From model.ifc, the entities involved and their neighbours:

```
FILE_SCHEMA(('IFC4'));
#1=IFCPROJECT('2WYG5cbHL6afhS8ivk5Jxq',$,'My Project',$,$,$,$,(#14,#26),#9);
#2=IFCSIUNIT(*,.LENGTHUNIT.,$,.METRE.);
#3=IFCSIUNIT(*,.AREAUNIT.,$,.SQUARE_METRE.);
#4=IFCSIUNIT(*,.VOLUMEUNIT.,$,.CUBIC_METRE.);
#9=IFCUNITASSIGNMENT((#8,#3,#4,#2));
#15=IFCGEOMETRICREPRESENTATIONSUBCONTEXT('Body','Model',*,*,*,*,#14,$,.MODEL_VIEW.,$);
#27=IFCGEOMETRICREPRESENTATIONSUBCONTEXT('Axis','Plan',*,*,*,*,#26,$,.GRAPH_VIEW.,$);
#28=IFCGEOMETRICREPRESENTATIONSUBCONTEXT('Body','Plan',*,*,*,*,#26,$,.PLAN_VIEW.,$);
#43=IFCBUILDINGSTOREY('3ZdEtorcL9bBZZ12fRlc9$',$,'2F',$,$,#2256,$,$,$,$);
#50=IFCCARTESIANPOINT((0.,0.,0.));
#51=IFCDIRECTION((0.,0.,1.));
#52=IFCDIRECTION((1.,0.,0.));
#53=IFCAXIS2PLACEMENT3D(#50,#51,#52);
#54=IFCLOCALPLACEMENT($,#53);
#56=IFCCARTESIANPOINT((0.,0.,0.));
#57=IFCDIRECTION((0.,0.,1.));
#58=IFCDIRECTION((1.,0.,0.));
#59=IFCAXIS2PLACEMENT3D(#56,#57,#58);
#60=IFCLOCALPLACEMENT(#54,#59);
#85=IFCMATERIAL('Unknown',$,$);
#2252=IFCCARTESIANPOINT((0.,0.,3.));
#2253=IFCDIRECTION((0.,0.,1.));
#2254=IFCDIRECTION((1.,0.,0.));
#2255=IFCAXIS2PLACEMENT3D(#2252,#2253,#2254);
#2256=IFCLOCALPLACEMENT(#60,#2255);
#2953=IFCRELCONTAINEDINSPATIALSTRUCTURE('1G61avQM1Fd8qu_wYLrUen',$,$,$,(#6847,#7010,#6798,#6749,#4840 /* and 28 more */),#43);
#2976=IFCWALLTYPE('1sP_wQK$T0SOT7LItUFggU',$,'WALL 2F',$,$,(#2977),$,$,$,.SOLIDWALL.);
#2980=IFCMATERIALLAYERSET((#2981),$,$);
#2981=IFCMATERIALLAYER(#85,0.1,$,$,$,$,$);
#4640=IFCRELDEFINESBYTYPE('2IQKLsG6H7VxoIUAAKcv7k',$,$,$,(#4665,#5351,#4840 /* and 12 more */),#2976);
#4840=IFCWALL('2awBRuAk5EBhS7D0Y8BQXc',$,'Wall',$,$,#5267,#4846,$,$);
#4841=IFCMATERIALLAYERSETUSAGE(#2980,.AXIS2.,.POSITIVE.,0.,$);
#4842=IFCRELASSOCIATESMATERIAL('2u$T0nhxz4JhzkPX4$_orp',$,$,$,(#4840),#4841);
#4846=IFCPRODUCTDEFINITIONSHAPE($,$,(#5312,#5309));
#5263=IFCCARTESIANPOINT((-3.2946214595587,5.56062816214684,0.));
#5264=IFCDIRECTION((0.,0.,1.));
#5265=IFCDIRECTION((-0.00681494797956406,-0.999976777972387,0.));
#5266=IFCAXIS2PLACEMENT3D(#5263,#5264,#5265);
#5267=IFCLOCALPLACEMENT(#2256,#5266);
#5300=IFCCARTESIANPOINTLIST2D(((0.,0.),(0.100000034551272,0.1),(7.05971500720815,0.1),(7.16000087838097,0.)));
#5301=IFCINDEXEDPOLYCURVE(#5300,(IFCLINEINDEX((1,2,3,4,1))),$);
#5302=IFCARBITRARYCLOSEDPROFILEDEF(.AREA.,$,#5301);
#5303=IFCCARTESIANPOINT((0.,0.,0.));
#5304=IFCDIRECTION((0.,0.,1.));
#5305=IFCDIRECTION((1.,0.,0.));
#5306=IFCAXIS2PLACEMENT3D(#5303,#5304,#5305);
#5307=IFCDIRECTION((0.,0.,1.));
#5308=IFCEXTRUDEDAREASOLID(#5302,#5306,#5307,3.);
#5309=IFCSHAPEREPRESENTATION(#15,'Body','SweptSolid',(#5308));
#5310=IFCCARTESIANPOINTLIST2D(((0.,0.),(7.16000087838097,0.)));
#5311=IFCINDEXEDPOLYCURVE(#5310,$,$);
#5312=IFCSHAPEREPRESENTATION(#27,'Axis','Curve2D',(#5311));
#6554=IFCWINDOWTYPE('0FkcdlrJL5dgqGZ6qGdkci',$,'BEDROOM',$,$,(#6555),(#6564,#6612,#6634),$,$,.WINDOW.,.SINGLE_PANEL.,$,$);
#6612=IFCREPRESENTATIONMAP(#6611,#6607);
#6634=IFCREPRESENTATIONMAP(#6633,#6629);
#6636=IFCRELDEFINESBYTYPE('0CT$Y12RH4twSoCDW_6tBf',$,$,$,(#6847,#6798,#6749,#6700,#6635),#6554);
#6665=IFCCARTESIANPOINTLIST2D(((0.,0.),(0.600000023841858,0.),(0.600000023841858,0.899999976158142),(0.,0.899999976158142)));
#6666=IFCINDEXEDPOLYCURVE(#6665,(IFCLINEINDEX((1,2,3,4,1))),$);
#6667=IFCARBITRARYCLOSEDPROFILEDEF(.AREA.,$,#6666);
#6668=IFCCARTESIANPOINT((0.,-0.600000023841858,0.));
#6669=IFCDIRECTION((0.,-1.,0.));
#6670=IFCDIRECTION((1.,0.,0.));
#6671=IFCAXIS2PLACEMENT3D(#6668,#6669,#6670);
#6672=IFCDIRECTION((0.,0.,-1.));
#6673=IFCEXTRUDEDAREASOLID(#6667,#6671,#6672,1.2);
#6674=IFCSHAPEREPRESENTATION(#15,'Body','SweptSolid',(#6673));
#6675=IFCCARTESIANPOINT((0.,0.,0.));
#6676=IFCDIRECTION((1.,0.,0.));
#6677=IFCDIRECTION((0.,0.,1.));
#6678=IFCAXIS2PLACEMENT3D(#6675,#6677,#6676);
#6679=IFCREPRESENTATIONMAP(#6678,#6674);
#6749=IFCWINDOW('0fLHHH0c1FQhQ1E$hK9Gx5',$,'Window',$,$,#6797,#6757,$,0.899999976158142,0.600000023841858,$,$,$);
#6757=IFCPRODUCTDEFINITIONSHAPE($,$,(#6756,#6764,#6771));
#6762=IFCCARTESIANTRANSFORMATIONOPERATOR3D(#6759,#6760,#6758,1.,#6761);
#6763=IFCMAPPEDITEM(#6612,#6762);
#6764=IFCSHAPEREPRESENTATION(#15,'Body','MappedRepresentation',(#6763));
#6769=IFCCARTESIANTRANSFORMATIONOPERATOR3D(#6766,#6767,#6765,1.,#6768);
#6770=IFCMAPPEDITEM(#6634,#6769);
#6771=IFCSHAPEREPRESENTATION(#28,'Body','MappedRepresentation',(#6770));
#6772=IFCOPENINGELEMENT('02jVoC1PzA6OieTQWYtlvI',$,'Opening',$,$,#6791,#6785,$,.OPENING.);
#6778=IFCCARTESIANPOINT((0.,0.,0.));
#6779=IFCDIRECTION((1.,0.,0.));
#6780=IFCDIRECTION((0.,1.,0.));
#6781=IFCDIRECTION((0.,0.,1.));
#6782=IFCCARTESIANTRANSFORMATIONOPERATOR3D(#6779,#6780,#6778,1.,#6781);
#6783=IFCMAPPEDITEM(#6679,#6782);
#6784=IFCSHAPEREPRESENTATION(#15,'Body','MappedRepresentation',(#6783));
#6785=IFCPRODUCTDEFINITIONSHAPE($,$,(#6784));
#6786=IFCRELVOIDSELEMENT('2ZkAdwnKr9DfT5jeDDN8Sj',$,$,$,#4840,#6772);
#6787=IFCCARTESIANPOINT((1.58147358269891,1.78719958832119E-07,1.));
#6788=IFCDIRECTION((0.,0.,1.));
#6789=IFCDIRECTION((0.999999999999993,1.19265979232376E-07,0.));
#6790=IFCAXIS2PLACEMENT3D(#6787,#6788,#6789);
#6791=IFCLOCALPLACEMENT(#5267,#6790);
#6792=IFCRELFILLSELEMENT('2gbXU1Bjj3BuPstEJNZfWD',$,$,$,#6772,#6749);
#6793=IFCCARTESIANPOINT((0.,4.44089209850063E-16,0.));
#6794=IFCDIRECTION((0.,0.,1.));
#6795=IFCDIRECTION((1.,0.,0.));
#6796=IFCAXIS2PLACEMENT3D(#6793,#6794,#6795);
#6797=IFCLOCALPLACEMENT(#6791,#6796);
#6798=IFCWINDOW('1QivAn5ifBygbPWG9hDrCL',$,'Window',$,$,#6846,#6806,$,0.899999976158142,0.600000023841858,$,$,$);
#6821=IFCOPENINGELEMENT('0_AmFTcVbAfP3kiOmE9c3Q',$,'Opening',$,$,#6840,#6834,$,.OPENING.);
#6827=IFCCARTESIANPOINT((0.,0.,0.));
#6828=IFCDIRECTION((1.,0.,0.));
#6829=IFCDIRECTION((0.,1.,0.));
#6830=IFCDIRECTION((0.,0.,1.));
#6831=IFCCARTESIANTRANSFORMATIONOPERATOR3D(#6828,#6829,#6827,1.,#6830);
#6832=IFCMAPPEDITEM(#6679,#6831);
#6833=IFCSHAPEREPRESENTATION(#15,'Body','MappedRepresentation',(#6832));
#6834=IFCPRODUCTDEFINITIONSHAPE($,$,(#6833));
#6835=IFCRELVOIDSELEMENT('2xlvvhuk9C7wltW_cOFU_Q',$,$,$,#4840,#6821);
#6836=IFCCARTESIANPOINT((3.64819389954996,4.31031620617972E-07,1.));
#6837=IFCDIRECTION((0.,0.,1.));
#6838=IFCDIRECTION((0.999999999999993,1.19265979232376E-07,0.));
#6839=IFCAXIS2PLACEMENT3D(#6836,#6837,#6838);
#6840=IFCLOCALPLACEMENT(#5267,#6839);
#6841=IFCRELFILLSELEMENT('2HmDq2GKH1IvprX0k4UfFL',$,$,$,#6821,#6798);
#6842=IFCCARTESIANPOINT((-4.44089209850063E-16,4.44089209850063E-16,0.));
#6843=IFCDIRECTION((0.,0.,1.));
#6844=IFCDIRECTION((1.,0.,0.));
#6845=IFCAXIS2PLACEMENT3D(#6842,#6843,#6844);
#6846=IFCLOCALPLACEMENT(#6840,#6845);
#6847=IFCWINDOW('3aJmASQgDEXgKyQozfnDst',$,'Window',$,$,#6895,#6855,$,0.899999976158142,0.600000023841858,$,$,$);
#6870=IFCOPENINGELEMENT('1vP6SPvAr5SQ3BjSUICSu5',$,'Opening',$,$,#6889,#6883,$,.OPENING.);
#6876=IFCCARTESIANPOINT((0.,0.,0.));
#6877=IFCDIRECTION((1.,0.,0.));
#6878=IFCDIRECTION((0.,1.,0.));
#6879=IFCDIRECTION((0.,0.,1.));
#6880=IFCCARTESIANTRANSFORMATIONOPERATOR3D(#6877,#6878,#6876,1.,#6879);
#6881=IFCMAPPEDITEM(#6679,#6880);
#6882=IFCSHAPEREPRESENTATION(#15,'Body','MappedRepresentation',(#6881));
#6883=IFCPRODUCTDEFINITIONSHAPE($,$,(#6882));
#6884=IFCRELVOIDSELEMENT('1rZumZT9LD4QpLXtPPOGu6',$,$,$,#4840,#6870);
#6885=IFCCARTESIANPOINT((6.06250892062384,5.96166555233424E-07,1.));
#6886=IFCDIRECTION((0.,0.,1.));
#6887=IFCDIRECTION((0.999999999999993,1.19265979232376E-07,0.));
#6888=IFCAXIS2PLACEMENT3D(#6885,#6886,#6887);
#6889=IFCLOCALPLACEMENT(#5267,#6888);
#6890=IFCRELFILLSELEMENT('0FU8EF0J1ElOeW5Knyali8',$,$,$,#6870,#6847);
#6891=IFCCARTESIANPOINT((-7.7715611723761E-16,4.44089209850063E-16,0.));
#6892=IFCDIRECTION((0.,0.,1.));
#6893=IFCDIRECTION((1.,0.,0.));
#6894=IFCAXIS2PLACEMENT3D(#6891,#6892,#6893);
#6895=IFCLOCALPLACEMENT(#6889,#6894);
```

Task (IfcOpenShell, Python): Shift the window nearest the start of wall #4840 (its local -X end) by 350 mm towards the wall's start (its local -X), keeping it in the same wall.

```python
import ifcopenshell
import ifcopenshell.api.geometry
import ifcopenshell.util.placement

model = ifcopenshell.open("model.ifc")

window = model.by_id(6749)
opening = window.FillsVoids[0].RelatingOpeningElement
wall = opening.VoidsElements[0].RelatingBuildingElement

wall_matrix = ifcopenshell.util.placement.get_local_placement(wall.ObjectPlacement)
shift = wall_matrix[:3, 0] * -0.35
before = ifcopenshell.util.placement.get_local_placement(window.ObjectPlacement)[:3, 3].copy()

# The window is placed relative to its opening, so it follows when the opening moves.
matrix = ifcopenshell.util.placement.get_local_placement(opening.ObjectPlacement)
matrix[:3, 3] += shift
ifcopenshell.api.geometry.edit_object_placement(
    model, product=opening, matrix=matrix, is_si=False, should_transform_children=True
)

after = ifcopenshell.util.placement.get_local_placement(window.ObjectPlacement)[:3, 3]
print("window moved by", (after - before).round(3) + 0.0)

model.write("model_v2.ifc")
```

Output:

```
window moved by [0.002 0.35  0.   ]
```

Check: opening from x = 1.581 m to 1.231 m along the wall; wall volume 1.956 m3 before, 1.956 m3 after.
